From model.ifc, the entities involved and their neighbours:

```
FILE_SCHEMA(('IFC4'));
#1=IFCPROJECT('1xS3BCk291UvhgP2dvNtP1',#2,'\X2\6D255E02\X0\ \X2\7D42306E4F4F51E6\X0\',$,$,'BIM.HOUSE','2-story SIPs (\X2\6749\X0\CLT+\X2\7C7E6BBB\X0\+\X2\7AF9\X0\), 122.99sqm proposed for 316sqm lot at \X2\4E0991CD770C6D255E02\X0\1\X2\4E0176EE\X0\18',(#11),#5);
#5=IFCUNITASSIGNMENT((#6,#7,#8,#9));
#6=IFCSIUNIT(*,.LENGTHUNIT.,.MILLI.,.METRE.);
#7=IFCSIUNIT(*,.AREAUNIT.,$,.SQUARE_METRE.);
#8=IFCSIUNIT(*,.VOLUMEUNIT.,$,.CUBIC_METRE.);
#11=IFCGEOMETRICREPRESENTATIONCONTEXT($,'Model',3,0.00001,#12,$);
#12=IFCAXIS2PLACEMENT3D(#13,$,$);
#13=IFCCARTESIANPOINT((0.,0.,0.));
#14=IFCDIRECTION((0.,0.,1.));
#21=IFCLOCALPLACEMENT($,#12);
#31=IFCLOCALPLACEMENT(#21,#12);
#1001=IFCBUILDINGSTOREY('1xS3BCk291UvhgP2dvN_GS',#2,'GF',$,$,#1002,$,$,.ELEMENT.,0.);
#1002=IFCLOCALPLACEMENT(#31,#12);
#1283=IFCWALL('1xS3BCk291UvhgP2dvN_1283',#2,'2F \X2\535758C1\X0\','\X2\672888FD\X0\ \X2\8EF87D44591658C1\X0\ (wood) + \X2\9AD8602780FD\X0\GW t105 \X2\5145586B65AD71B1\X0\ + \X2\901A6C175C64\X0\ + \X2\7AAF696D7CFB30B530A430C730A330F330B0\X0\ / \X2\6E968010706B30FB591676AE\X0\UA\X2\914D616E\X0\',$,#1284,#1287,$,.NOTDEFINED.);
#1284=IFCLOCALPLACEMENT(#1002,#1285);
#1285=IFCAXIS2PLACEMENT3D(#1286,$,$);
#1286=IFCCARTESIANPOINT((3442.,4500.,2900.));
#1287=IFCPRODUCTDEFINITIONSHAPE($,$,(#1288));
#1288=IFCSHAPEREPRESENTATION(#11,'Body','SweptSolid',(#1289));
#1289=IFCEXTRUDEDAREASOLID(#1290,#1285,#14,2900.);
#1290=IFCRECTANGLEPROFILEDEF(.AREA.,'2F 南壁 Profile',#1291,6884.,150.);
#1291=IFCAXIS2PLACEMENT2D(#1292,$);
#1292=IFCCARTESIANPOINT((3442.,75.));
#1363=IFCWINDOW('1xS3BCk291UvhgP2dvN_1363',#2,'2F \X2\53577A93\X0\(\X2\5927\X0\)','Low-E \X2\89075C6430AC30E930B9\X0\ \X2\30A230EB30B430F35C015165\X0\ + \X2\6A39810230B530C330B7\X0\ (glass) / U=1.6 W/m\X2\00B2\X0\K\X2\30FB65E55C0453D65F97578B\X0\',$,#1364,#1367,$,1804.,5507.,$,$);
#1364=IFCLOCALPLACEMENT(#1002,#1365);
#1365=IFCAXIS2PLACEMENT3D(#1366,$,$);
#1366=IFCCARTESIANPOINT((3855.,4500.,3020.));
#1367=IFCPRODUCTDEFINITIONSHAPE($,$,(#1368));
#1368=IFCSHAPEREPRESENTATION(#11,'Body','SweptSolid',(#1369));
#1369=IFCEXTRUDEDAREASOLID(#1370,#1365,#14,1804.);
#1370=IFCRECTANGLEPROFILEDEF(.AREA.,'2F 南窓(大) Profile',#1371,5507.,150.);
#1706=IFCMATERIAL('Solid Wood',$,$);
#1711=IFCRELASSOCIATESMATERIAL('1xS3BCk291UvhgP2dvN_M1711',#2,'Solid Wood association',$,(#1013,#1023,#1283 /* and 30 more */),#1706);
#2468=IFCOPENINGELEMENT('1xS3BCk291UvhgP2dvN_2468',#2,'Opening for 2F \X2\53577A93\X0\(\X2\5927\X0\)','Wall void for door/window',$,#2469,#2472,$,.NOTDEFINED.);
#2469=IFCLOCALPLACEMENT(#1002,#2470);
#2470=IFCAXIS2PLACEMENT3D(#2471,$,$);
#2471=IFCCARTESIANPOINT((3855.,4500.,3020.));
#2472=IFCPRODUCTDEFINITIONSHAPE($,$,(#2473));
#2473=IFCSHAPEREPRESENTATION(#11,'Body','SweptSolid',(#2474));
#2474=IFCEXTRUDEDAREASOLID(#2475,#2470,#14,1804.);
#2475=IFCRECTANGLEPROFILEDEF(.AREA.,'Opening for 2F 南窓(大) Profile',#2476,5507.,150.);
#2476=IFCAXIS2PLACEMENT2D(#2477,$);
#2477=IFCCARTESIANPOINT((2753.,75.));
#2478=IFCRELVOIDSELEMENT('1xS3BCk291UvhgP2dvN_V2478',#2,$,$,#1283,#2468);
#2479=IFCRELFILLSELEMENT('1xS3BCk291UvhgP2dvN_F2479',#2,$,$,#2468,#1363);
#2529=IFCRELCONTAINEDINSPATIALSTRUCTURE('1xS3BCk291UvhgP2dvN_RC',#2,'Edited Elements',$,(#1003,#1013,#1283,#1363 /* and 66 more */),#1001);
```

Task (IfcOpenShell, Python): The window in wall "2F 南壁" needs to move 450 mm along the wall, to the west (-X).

```python
import ifcopenshell
import ifcopenshell.api.geometry
import ifcopenshell.util.placement

model = ifcopenshell.open("model.ifc")

window = model.by_guid("1xS3BCk291UvhgP2dvN_1363")
opening = window.FillsVoids[0].RelatingOpeningElement
wall = opening.VoidsElements[0].RelatingBuildingElement

wall_matrix = ifcopenshell.util.placement.get_local_placement(wall.ObjectPlacement)
shift = wall_matrix[:3, 0] * -450.0
before = ifcopenshell.util.placement.get_local_placement(window.ObjectPlacement)[:3, 3].copy()

# The window is not placed relative to its opening, so move both.
for product in (opening, window):
    matrix = ifcopenshell.util.placement.get_local_placement(product.ObjectPlacement)
    matrix[:3, 3] += shift
    ifcopenshell.api.geometry.edit_object_placement(model, product=product, matrix=matrix, is_si=False)

after = ifcopenshell.util.placement.get_local_placement(window.ObjectPlacement)[:3, 3]
print("window moved by", (after - before).round(3) + 0.0)

model.write("model_v2.ifc")
```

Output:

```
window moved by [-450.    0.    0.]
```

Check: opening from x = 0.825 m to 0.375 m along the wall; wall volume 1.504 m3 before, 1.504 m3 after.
